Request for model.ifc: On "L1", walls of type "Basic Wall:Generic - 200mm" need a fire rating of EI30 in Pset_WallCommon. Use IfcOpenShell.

First a look at what the model holds.

```python
import ifcopenshell
import ifcopenshell.util.element

model = ifcopenshell.open("model.ifc")
print(model.schema)
storey = next(s for s in model.by_type("IfcBuildingStorey") if s.Name == "L1")
walls = [e for e in ifcopenshell.util.element.get_decomposition(storey) if e.is_a("IfcWall")]
seen = {}
for e in walls:
    element_type = ifcopenshell.util.element.get_type(e)
    key = (element_type.Name if element_type != e and element_type else None, ifcopenshell.util.element.get_pset(e, "Pset_WallCommon", "FireRating"))
    seen[key] = seen.get(key, 0) + 1
for (name, value), count in sorted(seen.items(), key=str):
    print(count, "x", name, "|", value)
```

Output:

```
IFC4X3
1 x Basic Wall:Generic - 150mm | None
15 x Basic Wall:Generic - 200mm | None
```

```python
import ifcopenshell
import ifcopenshell.api.pset
import ifcopenshell.util.element

model = ifcopenshell.open("model.ifc")

storey = next(s for s in model.by_type("IfcBuildingStorey") if s.Name == "L1")
walls = [e for e in ifcopenshell.util.element.get_decomposition(storey) if e.is_a("IfcWall")]

count = 0
for e in walls:
    element_type = ifcopenshell.util.element.get_type(e)
    if element_type in (None, e) or element_type.Name != "Basic Wall:Generic - 200mm":
        continue
    # add_pset returns the element's existing set when there is one.
    pset = ifcopenshell.api.pset.add_pset(model, product=e, name="Pset_WallCommon")
    ifcopenshell.api.pset.edit_pset(model, pset=pset, properties={"FireRating": "EI30"})
    count += 1

print(count, "walls updated")

model.write("model_rev.ifc")
```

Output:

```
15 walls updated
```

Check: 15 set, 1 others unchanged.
